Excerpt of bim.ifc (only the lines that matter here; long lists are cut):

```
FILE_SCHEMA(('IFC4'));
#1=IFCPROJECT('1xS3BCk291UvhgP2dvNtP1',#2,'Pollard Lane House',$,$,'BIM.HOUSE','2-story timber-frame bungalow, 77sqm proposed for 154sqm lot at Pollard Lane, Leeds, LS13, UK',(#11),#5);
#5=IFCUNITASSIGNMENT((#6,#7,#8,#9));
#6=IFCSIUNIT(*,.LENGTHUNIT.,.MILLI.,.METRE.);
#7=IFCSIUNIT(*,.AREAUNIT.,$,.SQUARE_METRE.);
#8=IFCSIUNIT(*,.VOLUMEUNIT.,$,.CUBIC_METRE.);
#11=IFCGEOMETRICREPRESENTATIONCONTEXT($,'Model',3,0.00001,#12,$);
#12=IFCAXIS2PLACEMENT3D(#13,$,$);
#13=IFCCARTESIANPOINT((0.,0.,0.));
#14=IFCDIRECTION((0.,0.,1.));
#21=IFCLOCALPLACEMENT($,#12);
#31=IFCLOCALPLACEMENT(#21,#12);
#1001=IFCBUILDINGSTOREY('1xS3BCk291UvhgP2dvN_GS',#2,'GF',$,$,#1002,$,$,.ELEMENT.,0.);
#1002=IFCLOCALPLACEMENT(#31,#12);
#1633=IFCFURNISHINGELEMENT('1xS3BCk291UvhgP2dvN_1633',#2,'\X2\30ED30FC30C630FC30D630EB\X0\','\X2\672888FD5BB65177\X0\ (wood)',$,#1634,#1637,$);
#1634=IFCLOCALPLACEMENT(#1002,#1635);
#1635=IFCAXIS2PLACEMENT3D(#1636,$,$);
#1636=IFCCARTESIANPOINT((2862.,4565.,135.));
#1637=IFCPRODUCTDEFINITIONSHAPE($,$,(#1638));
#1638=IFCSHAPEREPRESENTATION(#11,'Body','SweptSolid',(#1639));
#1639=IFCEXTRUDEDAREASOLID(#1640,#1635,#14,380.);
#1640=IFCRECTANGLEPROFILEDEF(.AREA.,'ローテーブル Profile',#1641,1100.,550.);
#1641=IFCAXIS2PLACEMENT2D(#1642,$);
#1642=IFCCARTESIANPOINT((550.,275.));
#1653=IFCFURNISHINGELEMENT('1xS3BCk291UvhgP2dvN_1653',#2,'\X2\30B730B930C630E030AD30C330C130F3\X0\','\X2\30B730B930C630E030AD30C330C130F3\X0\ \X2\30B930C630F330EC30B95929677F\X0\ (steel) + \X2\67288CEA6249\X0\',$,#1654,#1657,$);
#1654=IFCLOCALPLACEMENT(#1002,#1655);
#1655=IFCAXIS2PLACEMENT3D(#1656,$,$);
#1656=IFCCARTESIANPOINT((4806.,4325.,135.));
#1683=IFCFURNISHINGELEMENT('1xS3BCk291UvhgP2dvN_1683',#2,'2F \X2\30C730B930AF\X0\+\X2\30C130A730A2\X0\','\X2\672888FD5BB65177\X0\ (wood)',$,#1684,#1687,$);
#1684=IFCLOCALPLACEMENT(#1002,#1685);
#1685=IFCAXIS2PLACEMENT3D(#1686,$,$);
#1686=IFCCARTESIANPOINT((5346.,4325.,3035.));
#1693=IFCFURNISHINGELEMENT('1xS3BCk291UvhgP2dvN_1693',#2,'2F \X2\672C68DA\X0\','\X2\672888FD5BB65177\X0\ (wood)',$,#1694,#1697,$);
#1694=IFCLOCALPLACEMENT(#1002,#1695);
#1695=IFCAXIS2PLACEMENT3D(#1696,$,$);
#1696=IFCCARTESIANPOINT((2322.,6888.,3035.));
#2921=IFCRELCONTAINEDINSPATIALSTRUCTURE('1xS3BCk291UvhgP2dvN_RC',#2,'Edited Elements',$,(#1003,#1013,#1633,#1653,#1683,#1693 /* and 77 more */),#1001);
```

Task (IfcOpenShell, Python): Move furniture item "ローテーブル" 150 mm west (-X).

```python
import ifcopenshell
import ifcopenshell.api.geometry
import ifcopenshell.util.placement
import ifcopenshell.util.unit

model = ifcopenshell.open("bim.ifc")
unit_scale = ifcopenshell.util.unit.calculate_unit_scale(model)

item = model.by_id(1633)
matrix = ifcopenshell.util.placement.get_local_placement(item.ObjectPlacement)
matrix[0, 3] -= 0.15 / unit_scale
ifcopenshell.api.geometry.edit_object_placement(model, product=item, matrix=matrix, is_si=False)

print(ifcopenshell.util.placement.get_local_placement(item.ObjectPlacement).round(3) + 0.0)

model.write("bim_edited.ifc")
```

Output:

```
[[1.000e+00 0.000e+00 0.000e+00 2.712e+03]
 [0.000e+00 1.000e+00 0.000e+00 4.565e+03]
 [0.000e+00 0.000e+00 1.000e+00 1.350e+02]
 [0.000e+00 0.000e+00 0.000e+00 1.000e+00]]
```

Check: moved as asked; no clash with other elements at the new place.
